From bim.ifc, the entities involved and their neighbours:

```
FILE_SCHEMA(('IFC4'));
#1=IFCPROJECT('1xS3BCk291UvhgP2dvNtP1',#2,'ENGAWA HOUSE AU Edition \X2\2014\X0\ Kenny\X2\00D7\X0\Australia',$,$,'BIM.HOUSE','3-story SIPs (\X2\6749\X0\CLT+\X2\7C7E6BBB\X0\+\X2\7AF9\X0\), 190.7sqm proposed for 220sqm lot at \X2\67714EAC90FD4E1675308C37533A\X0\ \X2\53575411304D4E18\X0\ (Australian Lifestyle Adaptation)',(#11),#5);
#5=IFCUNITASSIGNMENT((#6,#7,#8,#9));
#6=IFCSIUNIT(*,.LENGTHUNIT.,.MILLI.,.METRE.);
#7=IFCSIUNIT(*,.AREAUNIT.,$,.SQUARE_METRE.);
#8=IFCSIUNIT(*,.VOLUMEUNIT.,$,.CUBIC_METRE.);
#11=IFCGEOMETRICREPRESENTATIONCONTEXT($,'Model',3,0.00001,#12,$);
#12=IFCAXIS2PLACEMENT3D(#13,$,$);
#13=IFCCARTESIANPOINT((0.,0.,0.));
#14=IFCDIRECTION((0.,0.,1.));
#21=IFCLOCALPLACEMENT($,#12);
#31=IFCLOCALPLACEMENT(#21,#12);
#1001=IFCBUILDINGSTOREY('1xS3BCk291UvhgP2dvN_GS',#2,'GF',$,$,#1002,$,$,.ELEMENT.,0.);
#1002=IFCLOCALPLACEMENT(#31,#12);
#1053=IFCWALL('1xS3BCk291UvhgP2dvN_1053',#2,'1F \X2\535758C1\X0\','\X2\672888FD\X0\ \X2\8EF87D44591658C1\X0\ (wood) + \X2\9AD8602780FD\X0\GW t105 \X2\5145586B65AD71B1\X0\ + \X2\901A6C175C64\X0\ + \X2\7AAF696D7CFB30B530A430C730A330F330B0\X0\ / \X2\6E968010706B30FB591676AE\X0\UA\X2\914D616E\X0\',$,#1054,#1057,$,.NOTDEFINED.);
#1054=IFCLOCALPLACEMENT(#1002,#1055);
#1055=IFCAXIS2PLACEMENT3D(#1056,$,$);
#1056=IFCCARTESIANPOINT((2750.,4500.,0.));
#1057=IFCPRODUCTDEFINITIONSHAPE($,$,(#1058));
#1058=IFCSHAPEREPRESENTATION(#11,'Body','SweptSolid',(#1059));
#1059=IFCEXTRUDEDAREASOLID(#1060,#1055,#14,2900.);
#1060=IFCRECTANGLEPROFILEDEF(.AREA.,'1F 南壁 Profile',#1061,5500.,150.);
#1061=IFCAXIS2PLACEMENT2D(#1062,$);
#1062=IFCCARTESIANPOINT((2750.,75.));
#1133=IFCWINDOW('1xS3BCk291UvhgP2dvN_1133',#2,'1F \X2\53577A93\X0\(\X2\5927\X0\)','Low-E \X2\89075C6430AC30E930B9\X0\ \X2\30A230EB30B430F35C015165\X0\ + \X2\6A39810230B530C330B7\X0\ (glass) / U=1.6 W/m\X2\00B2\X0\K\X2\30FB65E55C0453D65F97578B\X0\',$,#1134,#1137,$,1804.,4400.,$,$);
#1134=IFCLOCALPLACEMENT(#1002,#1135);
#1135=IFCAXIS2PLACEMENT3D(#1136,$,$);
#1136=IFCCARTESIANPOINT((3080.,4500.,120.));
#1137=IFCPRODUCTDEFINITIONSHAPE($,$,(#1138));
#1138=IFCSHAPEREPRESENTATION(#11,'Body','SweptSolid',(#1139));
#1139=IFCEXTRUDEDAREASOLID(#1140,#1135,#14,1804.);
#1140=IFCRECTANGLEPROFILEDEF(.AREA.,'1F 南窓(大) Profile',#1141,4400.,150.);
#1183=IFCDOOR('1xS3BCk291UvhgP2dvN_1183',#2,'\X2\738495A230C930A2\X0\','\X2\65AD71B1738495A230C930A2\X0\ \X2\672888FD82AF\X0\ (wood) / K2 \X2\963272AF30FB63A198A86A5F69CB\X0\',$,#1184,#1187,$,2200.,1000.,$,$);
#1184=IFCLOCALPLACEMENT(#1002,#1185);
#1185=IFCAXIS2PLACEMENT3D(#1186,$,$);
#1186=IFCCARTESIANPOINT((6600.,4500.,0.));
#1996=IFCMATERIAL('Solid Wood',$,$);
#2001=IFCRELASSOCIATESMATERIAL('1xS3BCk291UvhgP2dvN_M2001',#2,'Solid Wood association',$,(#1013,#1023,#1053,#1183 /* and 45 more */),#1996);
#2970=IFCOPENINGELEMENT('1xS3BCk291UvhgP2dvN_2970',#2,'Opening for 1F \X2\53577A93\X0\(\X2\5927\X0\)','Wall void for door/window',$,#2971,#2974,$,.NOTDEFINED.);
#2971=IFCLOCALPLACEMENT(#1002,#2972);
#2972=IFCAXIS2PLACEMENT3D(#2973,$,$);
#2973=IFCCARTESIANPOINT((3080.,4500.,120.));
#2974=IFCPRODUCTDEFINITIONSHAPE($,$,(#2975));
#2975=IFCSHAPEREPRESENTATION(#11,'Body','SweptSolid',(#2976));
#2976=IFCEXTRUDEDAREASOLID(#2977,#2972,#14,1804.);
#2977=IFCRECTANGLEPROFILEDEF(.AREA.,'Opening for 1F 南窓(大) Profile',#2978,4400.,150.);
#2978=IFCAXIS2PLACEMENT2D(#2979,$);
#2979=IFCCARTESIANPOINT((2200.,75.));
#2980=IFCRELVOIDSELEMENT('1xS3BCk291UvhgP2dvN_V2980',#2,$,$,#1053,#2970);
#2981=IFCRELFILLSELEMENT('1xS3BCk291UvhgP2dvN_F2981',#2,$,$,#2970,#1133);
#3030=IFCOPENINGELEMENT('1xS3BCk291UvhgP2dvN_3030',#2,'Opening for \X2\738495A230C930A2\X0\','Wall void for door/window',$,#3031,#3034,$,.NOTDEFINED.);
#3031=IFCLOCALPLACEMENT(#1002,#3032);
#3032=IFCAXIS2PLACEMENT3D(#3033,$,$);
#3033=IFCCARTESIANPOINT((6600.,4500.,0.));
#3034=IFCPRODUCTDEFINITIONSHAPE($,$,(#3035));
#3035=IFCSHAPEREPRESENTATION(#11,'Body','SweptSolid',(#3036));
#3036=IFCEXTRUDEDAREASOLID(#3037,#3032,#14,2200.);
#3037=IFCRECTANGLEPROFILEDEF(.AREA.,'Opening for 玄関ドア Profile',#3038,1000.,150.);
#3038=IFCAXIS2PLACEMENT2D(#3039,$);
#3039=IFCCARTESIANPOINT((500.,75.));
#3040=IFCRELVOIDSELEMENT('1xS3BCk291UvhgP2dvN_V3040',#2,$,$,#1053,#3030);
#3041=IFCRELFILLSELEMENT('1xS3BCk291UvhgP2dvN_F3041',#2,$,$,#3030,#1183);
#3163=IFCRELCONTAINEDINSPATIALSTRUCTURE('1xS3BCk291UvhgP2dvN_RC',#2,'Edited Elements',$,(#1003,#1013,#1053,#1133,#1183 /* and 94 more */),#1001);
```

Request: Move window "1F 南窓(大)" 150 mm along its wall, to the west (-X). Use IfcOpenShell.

```python
import ifcopenshell
import ifcopenshell.api.geometry
import ifcopenshell.util.placement
import ifcopenshell.util.unit

model = ifcopenshell.open("bim.ifc")
unit_scale = ifcopenshell.util.unit.calculate_unit_scale(model)

window = model.by_guid("1xS3BCk291UvhgP2dvN_1133")
opening = window.FillsVoids[0].RelatingOpeningElement
wall = opening.VoidsElements[0].RelatingBuildingElement

wall_matrix = ifcopenshell.util.placement.get_local_placement(wall.ObjectPlacement)
shift = wall_matrix[:3, 0] * -0.15 / unit_scale
before = ifcopenshell.util.placement.get_local_placement(window.ObjectPlacement)[:3, 3].copy()

# The window is not placed relative to its opening, so move both.
for product in (opening, window):
    matrix = ifcopenshell.util.placement.get_local_placement(product.ObjectPlacement)
    matrix[:3, 3] += shift
    ifcopenshell.api.geometry.edit_object_placement(model, product=product, matrix=matrix, is_si=False)

after = ifcopenshell.util.placement.get_local_placement(window.ObjectPlacement)[:3, 3]
print("window moved by", (after - before).round(3) + 0.0)

model.write("bim-out.ifc")
```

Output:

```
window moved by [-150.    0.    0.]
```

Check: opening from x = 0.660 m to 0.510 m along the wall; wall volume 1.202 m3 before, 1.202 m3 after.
